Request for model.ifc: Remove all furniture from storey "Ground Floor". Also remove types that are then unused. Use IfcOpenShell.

First a look at what the model holds.

```python
import ifcopenshell
import ifcopenshell.util.element

model = ifcopenshell.open("model.ifc")
print(model.schema)
storey = next(s for s in model.by_type("IfcBuildingStorey") if s.Name == "Ground Floor")
furniture = [e for e in ifcopenshell.util.element.get_decomposition(storey) if e.is_a("IfcFurnishingElement")]
seen = {}
for e in furniture:
    element_type = ifcopenshell.util.element.get_type(e)
    name = element_type.Name if element_type not in (None, e) else None
    seen[name] = seen.get(name, 0) + 1
for name, count in sorted(seen.items(), key=str):
    print(count, "x", name)
```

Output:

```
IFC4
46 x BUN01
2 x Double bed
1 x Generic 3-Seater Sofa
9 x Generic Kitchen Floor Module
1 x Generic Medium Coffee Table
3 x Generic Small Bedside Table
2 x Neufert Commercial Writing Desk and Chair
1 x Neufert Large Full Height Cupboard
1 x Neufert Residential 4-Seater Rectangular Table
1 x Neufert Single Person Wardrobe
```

```python
import ifcopenshell
import ifcopenshell.api.root
import ifcopenshell.util.element

model = ifcopenshell.open("model.ifc")

storey = next(s for s in model.by_type("IfcBuildingStorey") if s.Name == "Ground Floor")
furniture = [e for e in ifcopenshell.util.element.get_decomposition(storey) if e.is_a("IfcFurnishingElement")]
types = {ifcopenshell.util.element.get_type(e) for e in furniture} - {None, *furniture}

for e in furniture:
    ifcopenshell.api.root.remove_product(model, product=e)
print(len(furniture), "removed")

unused = [t for t in types if not ifcopenshell.util.element.get_types(t)]
for t in unused:
    ifcopenshell.api.root.remove_product(model, product=t)
print(len(unused), "unused types removed")

model.write("model_updated.ifc")
```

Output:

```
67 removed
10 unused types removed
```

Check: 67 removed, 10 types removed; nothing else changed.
